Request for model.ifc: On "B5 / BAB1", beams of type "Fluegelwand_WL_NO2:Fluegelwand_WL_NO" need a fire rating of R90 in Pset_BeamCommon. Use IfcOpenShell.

First a look at what the model holds.

```python
import ifcopenshell
import ifcopenshell.util.element

model = ifcopenshell.open("model.ifc")
print(model.schema)
storey = next(s for s in model.by_type("IfcBuildingStorey") if s.Name == "B5 / BAB1")
beams = [e for e in ifcopenshell.util.element.get_decomposition(storey) if e.is_a("IfcBeam")]
seen = {}
for e in beams:
    element_type = ifcopenshell.util.element.get_type(e)
    key = (element_type.Name if element_type != e and element_type else None, ifcopenshell.util.element.get_pset(e, "Pset_BeamCommon", "FireRating"))
    seen[key] = seen.get(key, 0) + 1
for (name, value), count in sorted(seen.items(), key=str):
    print(count, "x", name, "|", value)
```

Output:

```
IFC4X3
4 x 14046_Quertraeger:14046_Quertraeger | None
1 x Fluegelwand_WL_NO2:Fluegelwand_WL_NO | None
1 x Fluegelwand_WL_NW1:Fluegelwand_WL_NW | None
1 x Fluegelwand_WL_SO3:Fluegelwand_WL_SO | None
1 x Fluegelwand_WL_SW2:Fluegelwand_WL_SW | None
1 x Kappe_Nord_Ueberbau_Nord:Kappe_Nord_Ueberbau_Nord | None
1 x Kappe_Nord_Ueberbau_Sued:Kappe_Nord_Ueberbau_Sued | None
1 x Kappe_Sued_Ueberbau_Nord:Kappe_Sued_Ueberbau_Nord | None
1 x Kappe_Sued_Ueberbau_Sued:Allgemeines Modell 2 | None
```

```python
import ifcopenshell
import ifcopenshell.api.pset
import ifcopenshell.util.element

model = ifcopenshell.open("model.ifc")

storey = next(s for s in model.by_type("IfcBuildingStorey") if s.Name == "B5 / BAB1")
beams = [e for e in ifcopenshell.util.element.get_decomposition(storey) if e.is_a("IfcBeam")]

count = 0
for e in beams:
    element_type = ifcopenshell.util.element.get_type(e)
    if element_type in (None, e) or element_type.Name != "Fluegelwand_WL_NO2:Fluegelwand_WL_NO":
        continue
    # add_pset returns the element's existing set when there is one.
    pset = ifcopenshell.api.pset.add_pset(model, product=e, name="Pset_BeamCommon")
    ifcopenshell.api.pset.edit_pset(model, pset=pset, properties={"FireRating": "R90"})
    count += 1

print(count, "beams updated")

model.write("model_v2.ifc")
```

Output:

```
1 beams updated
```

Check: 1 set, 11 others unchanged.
